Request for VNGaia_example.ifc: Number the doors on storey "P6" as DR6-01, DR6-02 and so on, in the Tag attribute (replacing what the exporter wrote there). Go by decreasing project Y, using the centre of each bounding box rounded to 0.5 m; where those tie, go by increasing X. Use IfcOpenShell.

First a look at what the model holds.

```python
import ifcopenshell
import ifcopenshell.util.element
import ifcopenshell.util.placement

model = ifcopenshell.open("VNGaia_example.ifc")
print(model.schema)
storey = next(s for s in model.by_type("IfcBuildingStorey") if s.Name == "P6")
doors = [e for e in ifcopenshell.util.element.get_decomposition(storey) if e.is_a("IfcDoor")]
for e in sorted(doors, key=lambda e: e.id()):
    origin = ifcopenshell.util.placement.get_local_placement(e.ObjectPlacement)[:3, 3]
    print(e.id(), e.Tag, e.Name, origin.round(2) + 0.0, sep=" | ")
```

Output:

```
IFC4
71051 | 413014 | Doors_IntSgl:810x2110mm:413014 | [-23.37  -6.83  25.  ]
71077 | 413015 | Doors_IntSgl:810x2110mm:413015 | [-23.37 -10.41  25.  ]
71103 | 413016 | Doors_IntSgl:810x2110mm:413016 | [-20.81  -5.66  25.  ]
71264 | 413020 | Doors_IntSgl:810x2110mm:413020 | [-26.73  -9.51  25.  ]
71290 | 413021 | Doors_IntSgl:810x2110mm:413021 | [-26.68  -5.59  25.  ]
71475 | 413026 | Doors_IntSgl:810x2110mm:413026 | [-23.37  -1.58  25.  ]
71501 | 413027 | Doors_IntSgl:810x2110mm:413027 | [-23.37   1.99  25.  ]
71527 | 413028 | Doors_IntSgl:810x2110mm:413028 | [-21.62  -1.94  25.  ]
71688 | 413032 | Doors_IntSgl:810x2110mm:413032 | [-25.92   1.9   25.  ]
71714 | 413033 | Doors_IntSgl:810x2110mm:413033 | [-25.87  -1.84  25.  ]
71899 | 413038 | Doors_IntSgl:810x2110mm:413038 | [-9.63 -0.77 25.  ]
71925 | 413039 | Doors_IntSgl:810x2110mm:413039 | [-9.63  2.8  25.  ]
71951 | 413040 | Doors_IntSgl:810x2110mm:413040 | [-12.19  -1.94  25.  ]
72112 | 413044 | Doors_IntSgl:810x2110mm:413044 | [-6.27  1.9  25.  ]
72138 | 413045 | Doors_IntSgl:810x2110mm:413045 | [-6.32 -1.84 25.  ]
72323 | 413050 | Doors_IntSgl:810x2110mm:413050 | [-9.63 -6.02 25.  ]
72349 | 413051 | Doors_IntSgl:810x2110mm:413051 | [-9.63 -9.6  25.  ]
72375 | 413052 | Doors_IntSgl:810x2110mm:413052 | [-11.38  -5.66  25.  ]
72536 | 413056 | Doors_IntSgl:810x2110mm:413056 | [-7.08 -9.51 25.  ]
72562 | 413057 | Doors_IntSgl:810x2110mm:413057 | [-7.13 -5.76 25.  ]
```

```python
import ifcopenshell
import ifcopenshell.geom
import ifcopenshell.util.element
import ifcopenshell.util.shape

model = ifcopenshell.open("VNGaia_example.ifc")
settings = ifcopenshell.geom.settings()
settings.set("use-world-coords", True)


def centre(element):
    shape = ifcopenshell.geom.create_shape(settings, element)
    return ifcopenshell.util.shape.get_bbox_centroid(shape.geometry)


storey = next(s for s in model.by_type("IfcBuildingStorey") if s.Name == "P6")
doors = [e for e in ifcopenshell.util.element.get_decomposition(storey) if e.is_a("IfcDoor")]

# Insertion points can sit at a corner or the storey origin, so sort by the geometry (in metres).
centres = {e: centre(e) for e in doors}
doors.sort(key=lambda e: (-round(centres[e][1] / 0.5), centres[e][0]))

for i, e in enumerate(doors, start=1):
    number = f"DR6-{i:02d}"
    e.Tag = number
    print(e.id(), number)

model.write("VNGaia_example_rev.ifc")
```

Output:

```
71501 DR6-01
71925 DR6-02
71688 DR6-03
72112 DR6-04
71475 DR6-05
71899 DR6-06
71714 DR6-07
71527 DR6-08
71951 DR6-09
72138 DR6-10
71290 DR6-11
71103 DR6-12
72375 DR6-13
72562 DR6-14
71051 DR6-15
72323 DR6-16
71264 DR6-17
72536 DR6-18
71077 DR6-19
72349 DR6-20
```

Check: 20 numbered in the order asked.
